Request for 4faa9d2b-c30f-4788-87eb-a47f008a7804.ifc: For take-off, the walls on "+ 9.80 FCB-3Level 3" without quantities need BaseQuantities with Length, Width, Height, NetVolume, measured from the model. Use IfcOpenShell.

First a look at what the model holds.

```python
import ifcopenshell
import ifcopenshell.util.element
import ifcopenshell.util.unit

model = ifcopenshell.open("4faa9d2b-c30f-4788-87eb-a47f008a7804.ifc")
print(model.schema)
for unit_type in ("LENGTHUNIT", "AREAUNIT", "VOLUMEUNIT"):
    print(unit_type, ifcopenshell.util.unit.calculate_unit_scale(model, unit_type))
storey = next(s for s in model.by_type("IfcBuildingStorey") if s.Name == "+ 9.80 FCB-3Level 3")
walls = [e for e in ifcopenshell.util.element.get_decomposition(storey) if e.is_a("IfcWall")]
for e in sorted(walls, key=lambda e: e.id()):
    print(e.id(), e.is_a(), e.Name, list(ifcopenshell.util.element.get_psets(e, qtos_only=True)), sep=" | ")
```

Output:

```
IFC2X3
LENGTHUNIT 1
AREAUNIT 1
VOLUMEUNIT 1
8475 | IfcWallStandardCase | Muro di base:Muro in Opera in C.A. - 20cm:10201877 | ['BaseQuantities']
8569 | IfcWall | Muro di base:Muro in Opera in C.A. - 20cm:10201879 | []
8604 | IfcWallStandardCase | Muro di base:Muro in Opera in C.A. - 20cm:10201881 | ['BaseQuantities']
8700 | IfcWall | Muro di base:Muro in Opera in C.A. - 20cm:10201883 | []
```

```python
import ifcopenshell
import ifcopenshell.api.pset
import ifcopenshell.geom
import ifcopenshell.util.element
import ifcopenshell.util.shape
import ifcopenshell.util.unit

model = ifcopenshell.open("4faa9d2b-c30f-4788-87eb-a47f008a7804.ifc")
unit_scale = ifcopenshell.util.unit.calculate_unit_scale(model)
volume_scale = ifcopenshell.util.unit.calculate_unit_scale(model, "VOLUMEUNIT")
settings = ifcopenshell.geom.settings()

storey = next(s for s in model.by_type("IfcBuildingStorey") if s.Name == "+ 9.80 FCB-3Level 3")
walls = [e for e in ifcopenshell.util.element.get_decomposition(storey) if e.is_a("IfcWall")]

for e in sorted(walls, key=lambda e: e.id()):
    if ifcopenshell.util.element.get_psets(e, qtos_only=True, should_inherit=False):
        continue
    # Geometry comes back in metres, in the element's own axes.
    shape = ifcopenshell.geom.create_shape(settings, e)
    values = {
        "Length": ifcopenshell.util.shape.get_x(shape.geometry) / unit_scale,
        "Width": ifcopenshell.util.shape.get_y(shape.geometry) / unit_scale,
        "Height": ifcopenshell.util.shape.get_z(shape.geometry) / unit_scale,
        "NetVolume": ifcopenshell.util.shape.get_volume(shape.geometry) / volume_scale,
    }
    qto = ifcopenshell.api.pset.add_qto(model, product=e, name="BaseQuantities")
    ifcopenshell.api.pset.edit_qto(model, qto=qto, properties=values)
    print(e.id(), {k: round(v, 3) for k, v in values.items()})

model.write("4faa9d2b-c30f-4788-87eb-a47f008a7804-out.ifc")
```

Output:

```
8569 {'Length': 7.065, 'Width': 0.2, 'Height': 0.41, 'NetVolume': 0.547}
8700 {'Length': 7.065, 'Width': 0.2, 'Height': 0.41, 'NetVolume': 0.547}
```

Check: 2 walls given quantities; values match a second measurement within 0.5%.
